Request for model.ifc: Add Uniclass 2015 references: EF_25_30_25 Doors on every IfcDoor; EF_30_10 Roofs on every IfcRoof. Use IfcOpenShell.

First a look at what the model holds.

```python
import ifcopenshell

model = ifcopenshell.open("model.ifc")
print(model.schema)
print("classifications:", [c.Name for c in model.by_type("IfcClassification")])
for ifc_class in ("IfcDoor", "IfcRoof", "IfcStair", "IfcWall", "IfcWindow"):
    print(ifc_class, len(model.by_type(ifc_class)))
```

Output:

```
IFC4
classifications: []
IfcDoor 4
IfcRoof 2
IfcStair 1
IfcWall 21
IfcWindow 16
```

```python
import ifcopenshell
import ifcopenshell.api.classification

model = ifcopenshell.open("model.ifc")

system = ifcopenshell.api.classification.add_classification(model, classification="Uniclass 2015")

codes = {
    "IfcDoor": ("EF_25_30_25", "Doors"),
    "IfcRoof": ("EF_30_10", "Roofs"),
}
for ifc_class, (code, name) in codes.items():
    products = model.by_type(ifc_class)
    ifcopenshell.api.classification.add_reference(
        model, products=products, classification=system, identification=code, name=name
    )
    print(code, len(products))

model.write("model_updated.ifc")
```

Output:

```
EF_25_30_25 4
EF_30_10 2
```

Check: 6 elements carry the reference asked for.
